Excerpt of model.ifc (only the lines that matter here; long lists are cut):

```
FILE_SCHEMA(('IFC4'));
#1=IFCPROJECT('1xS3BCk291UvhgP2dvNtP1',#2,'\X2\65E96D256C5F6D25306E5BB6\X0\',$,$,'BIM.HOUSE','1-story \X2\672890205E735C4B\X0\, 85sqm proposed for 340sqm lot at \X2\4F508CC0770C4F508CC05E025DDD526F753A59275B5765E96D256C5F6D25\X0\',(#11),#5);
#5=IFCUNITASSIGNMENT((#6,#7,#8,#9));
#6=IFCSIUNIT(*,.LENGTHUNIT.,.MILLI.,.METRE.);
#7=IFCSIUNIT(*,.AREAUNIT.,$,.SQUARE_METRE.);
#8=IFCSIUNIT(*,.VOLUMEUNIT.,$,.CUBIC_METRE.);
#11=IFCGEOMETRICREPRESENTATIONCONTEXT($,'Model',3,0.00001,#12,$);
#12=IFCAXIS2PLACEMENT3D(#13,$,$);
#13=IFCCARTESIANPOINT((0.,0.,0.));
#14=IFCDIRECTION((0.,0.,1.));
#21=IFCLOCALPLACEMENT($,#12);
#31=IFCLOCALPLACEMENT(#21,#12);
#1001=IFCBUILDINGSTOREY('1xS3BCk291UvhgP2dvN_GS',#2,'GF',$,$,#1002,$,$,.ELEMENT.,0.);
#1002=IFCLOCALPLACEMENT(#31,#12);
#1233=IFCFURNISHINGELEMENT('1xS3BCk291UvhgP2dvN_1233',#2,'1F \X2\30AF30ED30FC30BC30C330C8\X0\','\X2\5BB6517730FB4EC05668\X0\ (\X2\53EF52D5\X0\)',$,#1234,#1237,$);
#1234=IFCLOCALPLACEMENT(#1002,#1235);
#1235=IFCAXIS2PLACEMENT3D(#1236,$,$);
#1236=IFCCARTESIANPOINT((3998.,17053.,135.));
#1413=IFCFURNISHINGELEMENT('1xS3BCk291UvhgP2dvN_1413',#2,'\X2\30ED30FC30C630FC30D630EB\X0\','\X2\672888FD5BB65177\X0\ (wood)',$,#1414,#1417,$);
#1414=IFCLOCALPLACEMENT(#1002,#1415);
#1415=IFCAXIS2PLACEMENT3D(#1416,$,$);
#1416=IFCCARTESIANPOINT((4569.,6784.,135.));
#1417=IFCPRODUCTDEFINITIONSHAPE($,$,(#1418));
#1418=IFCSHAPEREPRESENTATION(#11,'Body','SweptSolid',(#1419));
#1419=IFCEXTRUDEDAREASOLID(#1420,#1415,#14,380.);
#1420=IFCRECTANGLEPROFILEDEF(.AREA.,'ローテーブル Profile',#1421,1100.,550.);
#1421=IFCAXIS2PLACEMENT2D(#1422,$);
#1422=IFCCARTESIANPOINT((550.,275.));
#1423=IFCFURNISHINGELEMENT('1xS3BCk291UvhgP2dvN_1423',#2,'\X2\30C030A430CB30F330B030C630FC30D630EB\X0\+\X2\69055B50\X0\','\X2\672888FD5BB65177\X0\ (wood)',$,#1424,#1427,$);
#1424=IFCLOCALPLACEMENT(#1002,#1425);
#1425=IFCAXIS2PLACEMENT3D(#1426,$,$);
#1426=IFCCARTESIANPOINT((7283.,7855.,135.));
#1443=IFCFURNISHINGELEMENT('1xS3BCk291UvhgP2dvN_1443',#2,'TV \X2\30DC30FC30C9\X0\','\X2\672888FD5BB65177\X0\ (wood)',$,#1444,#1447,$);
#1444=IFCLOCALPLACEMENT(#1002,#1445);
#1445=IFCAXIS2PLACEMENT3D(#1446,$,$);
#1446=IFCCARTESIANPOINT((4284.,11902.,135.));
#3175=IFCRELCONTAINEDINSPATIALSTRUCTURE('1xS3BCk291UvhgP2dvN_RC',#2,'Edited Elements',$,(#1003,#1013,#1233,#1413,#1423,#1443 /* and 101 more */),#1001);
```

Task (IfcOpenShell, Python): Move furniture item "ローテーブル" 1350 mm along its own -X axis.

```python
import ifcopenshell
import ifcopenshell.api.geometry
import ifcopenshell.util.placement

model = ifcopenshell.open("model.ifc")

item = model.by_guid("1xS3BCk291UvhgP2dvN_1413")
matrix = ifcopenshell.util.placement.get_local_placement(item.ObjectPlacement)
matrix[:3, 3] -= matrix[:3, 0] * 1350.0
ifcopenshell.api.geometry.edit_object_placement(model, product=item, matrix=matrix, is_si=False)

print(ifcopenshell.util.placement.get_local_placement(item.ObjectPlacement).round(3) + 0.0)

model.write("model_v2.ifc")
```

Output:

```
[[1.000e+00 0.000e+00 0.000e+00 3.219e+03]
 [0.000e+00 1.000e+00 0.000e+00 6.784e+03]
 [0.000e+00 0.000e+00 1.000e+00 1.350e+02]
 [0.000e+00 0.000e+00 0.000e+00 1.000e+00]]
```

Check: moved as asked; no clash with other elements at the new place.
